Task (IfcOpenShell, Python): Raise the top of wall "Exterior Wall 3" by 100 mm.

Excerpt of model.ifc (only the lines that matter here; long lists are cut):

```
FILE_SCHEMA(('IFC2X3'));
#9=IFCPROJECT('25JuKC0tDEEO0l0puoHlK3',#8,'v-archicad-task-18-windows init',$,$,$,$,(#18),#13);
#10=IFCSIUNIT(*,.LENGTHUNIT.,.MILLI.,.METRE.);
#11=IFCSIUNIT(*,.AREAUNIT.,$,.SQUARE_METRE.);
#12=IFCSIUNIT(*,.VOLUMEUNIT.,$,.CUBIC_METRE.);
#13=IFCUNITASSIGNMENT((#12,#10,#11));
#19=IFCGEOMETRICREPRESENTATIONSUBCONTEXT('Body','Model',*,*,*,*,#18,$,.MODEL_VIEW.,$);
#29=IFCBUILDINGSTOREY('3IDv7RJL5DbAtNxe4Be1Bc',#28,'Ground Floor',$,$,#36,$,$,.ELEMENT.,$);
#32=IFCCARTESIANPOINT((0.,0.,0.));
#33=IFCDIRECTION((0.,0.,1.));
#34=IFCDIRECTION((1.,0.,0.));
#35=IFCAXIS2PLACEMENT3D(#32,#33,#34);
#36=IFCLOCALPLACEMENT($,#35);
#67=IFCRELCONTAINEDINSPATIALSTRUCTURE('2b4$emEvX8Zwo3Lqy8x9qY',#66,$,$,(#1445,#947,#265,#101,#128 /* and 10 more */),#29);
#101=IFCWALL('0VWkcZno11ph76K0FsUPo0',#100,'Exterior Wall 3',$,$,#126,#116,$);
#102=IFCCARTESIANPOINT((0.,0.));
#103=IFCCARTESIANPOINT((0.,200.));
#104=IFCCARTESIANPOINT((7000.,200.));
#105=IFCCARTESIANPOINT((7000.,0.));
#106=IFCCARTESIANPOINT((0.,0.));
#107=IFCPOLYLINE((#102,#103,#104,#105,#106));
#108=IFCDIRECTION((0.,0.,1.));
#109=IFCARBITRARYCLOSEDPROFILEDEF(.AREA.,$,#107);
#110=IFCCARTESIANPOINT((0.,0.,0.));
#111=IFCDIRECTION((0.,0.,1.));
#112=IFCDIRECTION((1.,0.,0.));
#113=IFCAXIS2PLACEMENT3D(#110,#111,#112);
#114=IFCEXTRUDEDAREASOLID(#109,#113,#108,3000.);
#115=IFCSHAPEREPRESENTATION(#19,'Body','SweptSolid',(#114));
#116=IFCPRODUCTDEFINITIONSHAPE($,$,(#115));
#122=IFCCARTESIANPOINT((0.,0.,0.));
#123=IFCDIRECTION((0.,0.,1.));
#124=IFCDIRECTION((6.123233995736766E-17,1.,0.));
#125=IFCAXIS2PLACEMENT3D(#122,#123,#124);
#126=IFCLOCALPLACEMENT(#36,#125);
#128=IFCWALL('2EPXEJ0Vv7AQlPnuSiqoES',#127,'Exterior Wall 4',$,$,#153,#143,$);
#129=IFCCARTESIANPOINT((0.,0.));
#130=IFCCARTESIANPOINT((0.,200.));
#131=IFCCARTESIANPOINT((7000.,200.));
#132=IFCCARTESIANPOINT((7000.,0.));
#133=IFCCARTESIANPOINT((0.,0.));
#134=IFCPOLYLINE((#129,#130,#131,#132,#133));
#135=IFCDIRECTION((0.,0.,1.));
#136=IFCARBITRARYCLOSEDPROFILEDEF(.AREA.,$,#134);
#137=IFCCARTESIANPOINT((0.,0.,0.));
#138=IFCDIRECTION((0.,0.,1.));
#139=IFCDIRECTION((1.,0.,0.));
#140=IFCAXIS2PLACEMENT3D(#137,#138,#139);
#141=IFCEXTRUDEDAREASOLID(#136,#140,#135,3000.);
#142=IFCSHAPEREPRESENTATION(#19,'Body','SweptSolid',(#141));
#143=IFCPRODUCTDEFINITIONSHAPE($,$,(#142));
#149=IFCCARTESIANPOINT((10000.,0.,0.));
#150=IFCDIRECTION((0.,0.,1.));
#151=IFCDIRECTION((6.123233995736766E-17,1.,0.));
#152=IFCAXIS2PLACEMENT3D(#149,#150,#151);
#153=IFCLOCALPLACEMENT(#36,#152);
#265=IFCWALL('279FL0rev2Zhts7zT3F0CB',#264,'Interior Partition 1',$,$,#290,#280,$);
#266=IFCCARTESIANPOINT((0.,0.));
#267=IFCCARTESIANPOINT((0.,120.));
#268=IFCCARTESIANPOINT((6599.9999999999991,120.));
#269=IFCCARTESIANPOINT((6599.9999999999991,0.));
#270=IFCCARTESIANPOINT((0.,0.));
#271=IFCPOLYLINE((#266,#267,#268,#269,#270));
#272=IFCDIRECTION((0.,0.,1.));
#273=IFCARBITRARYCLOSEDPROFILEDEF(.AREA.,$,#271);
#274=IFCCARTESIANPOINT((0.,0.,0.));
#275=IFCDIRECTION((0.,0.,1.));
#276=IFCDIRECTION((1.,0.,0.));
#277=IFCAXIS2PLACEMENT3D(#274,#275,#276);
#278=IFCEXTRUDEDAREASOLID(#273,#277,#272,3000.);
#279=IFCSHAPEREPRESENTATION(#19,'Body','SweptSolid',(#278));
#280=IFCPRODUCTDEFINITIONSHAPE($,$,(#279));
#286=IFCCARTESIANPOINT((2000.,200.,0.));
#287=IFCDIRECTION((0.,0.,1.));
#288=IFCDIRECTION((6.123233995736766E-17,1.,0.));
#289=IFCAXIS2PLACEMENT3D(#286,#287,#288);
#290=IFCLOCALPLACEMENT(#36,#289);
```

```python
import ifcopenshell
import ifcopenshell.geom
import ifcopenshell.util.representation
import ifcopenshell.util.shape
import ifcopenshell.util.unit

model = ifcopenshell.open("model.ifc")
unit_scale = ifcopenshell.util.unit.calculate_unit_scale(model)
settings = ifcopenshell.geom.settings()


def volume(element):
    """Net volume in cubic metres, openings subtracted."""
    shape = ifcopenshell.geom.create_shape(settings, element)
    return ifcopenshell.util.shape.get_volume(shape.geometry)


wall = model.by_id(101)
before = volume(wall)

body = ifcopenshell.util.representation.get_representation(wall, "Model", "Body")
solid = body.Items[0]
old_height = solid.Depth
solid.Depth += 0.1 / unit_scale
after = volume(wall)

print(f"height {old_height:g} -> {solid.Depth:g}, volume {before:.3f} -> {after:.3f} m3")

model.write("model-out.ifc")
```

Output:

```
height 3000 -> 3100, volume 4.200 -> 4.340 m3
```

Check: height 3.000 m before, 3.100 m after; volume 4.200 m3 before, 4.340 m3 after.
